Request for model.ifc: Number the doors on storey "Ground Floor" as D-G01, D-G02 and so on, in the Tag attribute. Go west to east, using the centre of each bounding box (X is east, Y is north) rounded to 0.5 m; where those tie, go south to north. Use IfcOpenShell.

First a look at what the model holds.

```python
import ifcopenshell
import ifcopenshell.util.element
import ifcopenshell.util.placement

model = ifcopenshell.open("model.ifc")
print(model.schema)
storey = next(s for s in model.by_type("IfcBuildingStorey") if s.Name == "Ground Floor")
doors = [e for e in ifcopenshell.util.element.get_decomposition(storey) if e.is_a("IfcDoor")]
for e in sorted(doors, key=lambda e: e.id()):
    origin = ifcopenshell.util.placement.get_local_placement(e.ObjectPlacement)[:3, 3]
    print(e.id(), e.Tag, e.Name, origin.round(2) + 0.0, sep=" | ")
```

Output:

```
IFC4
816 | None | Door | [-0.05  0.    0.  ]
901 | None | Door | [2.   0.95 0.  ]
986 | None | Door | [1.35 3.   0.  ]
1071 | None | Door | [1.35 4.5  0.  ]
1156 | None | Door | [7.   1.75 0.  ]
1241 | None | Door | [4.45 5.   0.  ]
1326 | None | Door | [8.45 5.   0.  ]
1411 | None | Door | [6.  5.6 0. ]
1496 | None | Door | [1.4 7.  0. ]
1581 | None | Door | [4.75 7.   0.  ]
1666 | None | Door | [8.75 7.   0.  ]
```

```python
import ifcopenshell
import ifcopenshell.geom
import ifcopenshell.util.element
import ifcopenshell.util.shape

model = ifcopenshell.open("model.ifc")
settings = ifcopenshell.geom.settings()
settings.set("use-world-coords", True)


def centre(element):
    shape = ifcopenshell.geom.create_shape(settings, element)
    return ifcopenshell.util.shape.get_bbox_centroid(shape.geometry)


storey = next(s for s in model.by_type("IfcBuildingStorey") if s.Name == "Ground Floor")
doors = [e for e in ifcopenshell.util.element.get_decomposition(storey) if e.is_a("IfcDoor")]

# Insertion points can sit at a corner or the storey origin, so sort by the geometry (in metres).
centres = {e: centre(e) for e in doors}
doors.sort(key=lambda e: (round(centres[e][0] / 0.5), centres[e][1]))

for i, e in enumerate(doors, start=1):
    number = f"D-G{i:02d}"
    e.Tag = number
    print(e.id(), number)

model.write("model_v2.ifc")
```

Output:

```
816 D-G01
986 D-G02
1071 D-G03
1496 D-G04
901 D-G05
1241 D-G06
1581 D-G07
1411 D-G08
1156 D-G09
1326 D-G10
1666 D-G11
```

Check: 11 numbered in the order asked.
